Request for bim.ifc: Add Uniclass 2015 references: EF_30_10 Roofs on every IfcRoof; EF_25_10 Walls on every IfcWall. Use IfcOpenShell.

First a look at what the model holds.

```python
import ifcopenshell

model = ifcopenshell.open("bim.ifc")
print(model.schema)
print("classifications:", [c.Name for c in model.by_type("IfcClassification")])
for ifc_class in ("IfcDoor", "IfcRoof", "IfcStair", "IfcWall", "IfcWindow"):
    print(ifc_class, len(model.by_type(ifc_class)))
```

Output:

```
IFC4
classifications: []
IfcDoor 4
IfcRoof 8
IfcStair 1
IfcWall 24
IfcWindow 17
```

```python
import ifcopenshell
import ifcopenshell.api.classification

model = ifcopenshell.open("bim.ifc")

system = ifcopenshell.api.classification.add_classification(model, classification="Uniclass 2015")

codes = {
    "IfcRoof": ("EF_30_10", "Roofs"),
    "IfcWall": ("EF_25_10", "Walls"),
}
for ifc_class, (code, name) in codes.items():
    products = model.by_type(ifc_class)
    ifcopenshell.api.classification.add_reference(
        model, products=products, classification=system, identification=code, name=name
    )
    print(code, len(products))

model.write("bim-out.ifc")
```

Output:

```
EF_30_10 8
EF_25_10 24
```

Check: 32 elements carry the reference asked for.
